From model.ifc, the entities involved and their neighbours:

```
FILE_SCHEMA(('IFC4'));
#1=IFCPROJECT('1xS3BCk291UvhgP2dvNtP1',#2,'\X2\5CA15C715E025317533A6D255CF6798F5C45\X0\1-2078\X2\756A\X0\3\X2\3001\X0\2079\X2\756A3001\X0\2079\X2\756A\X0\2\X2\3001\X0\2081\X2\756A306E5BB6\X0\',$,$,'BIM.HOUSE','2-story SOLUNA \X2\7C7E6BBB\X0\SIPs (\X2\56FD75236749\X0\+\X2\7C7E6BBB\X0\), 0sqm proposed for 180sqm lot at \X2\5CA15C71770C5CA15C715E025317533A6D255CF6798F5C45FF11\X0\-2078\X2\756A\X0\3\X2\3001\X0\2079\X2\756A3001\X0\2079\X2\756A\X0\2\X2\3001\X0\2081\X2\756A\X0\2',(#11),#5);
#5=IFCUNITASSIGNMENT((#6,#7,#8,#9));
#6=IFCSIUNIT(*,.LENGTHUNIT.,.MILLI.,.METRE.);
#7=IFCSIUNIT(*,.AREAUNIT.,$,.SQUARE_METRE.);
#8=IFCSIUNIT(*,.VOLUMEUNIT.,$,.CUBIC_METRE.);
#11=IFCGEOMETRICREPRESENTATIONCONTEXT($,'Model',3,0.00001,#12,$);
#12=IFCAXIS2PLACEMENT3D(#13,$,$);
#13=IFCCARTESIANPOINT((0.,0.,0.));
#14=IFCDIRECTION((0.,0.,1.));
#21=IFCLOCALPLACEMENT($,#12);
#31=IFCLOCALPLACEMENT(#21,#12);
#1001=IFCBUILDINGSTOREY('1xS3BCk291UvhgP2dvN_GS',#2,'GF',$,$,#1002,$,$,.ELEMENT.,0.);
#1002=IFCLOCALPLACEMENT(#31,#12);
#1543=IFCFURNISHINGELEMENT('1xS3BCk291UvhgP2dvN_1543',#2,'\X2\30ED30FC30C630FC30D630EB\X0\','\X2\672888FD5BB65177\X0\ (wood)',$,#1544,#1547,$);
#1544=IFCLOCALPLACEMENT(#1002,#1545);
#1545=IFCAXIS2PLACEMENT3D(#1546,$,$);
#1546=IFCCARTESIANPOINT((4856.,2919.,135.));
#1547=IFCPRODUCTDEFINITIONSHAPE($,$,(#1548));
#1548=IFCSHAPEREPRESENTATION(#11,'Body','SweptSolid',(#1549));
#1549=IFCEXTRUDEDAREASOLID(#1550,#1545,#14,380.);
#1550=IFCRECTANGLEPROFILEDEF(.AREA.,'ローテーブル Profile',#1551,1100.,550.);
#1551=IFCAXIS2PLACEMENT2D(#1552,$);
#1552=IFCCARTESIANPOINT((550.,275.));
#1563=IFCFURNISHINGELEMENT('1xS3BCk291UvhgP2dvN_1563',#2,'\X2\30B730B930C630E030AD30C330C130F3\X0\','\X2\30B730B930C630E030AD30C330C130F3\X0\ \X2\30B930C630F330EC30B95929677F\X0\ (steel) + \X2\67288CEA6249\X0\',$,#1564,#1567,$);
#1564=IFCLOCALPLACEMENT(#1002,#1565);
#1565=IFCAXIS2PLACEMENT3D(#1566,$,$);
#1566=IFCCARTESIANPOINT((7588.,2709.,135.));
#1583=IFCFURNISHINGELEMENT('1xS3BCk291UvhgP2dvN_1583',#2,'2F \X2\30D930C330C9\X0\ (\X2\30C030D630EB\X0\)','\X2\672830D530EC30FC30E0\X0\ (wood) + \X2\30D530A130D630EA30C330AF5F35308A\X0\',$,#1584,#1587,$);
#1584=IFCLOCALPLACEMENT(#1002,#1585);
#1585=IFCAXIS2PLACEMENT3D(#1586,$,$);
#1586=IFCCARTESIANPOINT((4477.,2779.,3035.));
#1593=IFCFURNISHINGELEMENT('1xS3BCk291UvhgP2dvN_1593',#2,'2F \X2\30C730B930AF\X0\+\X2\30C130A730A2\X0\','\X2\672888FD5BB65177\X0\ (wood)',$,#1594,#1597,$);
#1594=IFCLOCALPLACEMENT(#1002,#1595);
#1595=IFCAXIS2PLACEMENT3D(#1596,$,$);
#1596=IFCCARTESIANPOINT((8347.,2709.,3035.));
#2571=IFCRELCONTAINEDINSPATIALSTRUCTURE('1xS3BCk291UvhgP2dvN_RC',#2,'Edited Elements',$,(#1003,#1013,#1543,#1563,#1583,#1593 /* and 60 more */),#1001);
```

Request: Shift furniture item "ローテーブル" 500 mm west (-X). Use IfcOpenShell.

```python
import ifcopenshell
import ifcopenshell.api.geometry
import ifcopenshell.util.placement

model = ifcopenshell.open("model.ifc")

item = model.by_guid("1xS3BCk291UvhgP2dvN_1543")
matrix = ifcopenshell.util.placement.get_local_placement(item.ObjectPlacement)
matrix[0, 3] -= 500.0
ifcopenshell.api.geometry.edit_object_placement(model, product=item, matrix=matrix, is_si=False)

print(ifcopenshell.util.placement.get_local_placement(item.ObjectPlacement).round(3) + 0.0)

model.write("model_edited.ifc")
```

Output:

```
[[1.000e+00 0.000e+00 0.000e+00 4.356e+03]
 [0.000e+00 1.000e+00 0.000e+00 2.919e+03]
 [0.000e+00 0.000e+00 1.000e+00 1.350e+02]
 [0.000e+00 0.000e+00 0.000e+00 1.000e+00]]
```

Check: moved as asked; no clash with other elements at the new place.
